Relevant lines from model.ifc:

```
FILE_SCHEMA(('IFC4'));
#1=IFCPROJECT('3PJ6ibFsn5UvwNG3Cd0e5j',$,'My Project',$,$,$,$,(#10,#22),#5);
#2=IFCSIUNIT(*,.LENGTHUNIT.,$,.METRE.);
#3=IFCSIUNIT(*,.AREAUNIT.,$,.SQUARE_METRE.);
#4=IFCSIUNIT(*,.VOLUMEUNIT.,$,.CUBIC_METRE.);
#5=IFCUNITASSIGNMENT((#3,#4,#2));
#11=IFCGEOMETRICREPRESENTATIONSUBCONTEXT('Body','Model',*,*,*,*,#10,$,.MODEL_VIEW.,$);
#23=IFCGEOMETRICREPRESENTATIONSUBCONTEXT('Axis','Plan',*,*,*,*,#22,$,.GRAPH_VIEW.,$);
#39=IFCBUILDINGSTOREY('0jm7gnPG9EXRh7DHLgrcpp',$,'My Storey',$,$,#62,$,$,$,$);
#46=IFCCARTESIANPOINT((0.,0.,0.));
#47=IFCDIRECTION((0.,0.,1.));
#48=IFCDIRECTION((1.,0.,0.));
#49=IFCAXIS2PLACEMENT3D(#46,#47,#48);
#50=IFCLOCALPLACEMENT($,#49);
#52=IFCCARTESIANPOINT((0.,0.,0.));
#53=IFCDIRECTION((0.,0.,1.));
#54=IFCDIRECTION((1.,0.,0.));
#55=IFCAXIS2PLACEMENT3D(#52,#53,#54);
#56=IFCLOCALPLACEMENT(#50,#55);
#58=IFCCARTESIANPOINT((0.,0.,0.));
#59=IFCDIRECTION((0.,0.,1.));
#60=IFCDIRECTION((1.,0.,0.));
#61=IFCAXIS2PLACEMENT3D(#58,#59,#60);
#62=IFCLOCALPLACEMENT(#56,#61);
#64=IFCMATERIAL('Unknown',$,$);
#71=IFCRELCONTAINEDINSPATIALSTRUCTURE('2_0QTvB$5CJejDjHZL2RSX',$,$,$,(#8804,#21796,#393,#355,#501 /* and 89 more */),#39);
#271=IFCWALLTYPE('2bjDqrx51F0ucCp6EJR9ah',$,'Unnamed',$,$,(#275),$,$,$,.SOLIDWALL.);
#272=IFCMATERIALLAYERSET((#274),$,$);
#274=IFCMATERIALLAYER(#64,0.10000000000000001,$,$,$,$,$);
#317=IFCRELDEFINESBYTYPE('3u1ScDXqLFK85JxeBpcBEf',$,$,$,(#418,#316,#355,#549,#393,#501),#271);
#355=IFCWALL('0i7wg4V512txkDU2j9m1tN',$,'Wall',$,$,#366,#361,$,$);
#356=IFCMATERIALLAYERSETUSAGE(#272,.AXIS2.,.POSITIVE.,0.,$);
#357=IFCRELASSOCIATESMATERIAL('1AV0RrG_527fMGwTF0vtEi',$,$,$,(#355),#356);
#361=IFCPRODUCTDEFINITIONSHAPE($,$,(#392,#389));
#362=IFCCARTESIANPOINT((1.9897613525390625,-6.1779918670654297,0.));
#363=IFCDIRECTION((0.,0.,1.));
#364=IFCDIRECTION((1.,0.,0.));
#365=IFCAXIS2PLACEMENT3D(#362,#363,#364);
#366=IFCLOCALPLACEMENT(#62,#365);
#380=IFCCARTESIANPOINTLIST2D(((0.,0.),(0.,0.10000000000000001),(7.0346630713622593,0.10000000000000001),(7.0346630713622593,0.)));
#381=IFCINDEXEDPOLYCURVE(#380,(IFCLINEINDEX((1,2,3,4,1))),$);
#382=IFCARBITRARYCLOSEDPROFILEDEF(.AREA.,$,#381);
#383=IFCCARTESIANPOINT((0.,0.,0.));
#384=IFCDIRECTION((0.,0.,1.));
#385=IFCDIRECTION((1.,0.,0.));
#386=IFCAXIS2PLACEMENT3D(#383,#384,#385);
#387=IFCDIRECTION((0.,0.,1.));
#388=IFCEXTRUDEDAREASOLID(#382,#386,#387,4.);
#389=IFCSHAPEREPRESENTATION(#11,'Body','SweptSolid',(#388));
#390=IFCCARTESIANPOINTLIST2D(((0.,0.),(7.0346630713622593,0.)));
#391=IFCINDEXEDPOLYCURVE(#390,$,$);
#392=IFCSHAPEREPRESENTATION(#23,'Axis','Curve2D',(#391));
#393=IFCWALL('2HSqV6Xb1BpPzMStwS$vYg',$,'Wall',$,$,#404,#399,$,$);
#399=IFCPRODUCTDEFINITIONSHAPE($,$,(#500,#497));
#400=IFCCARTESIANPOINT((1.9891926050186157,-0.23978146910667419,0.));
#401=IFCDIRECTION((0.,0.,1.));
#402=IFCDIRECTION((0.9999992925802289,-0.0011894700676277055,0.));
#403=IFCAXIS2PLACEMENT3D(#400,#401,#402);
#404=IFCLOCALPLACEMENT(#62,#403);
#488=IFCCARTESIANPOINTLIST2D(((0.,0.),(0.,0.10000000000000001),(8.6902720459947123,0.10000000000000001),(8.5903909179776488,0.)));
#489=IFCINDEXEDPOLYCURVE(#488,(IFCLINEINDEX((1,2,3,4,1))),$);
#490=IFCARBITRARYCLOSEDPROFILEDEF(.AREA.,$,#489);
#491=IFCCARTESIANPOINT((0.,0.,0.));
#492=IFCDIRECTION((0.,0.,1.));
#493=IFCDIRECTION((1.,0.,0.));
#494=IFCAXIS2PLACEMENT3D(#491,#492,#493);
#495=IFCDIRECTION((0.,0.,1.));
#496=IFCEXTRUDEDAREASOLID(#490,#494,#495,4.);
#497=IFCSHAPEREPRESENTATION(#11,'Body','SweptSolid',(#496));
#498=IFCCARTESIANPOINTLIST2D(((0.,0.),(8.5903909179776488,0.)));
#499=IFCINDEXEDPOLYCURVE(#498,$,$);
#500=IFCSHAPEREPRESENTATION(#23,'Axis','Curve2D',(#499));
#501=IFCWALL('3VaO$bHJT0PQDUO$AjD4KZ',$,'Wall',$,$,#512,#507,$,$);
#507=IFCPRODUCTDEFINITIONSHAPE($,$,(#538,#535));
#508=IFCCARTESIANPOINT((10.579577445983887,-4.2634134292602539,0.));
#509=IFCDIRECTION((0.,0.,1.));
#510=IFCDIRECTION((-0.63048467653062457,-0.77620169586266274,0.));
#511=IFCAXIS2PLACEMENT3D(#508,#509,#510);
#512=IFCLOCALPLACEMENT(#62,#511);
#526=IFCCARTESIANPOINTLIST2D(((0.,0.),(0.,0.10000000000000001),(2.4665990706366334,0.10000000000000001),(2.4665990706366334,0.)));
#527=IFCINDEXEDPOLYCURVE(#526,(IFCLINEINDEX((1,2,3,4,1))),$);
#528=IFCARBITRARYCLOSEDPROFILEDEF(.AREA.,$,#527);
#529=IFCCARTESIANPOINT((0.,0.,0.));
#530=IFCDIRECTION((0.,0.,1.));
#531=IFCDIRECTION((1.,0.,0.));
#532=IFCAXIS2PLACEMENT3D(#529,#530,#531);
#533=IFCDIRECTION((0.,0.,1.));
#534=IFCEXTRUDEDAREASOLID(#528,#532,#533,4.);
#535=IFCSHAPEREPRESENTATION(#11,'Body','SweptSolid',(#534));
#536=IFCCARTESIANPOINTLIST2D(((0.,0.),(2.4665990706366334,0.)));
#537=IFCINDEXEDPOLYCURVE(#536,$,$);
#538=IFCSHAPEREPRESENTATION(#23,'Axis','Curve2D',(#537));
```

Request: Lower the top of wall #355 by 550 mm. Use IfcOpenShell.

```python
import ifcopenshell
import ifcopenshell.geom
import ifcopenshell.util.representation
import ifcopenshell.util.shape
import ifcopenshell.util.unit

model = ifcopenshell.open("model.ifc")
unit_scale = ifcopenshell.util.unit.calculate_unit_scale(model)
settings = ifcopenshell.geom.settings()


def volume(element):
    """Net volume in cubic metres, openings subtracted."""
    shape = ifcopenshell.geom.create_shape(settings, element)
    return ifcopenshell.util.shape.get_volume(shape.geometry)


wall = model.by_id(355)
before = volume(wall)

body = ifcopenshell.util.representation.get_representation(wall, "Model", "Body")
solid = body.Items[0]
old_height = solid.Depth
solid.Depth -= 0.55 / unit_scale
after = volume(wall)

print(f"height {old_height:g} -> {solid.Depth:g}, volume {before:.3f} -> {after:.3f} m3")

model.write("model-out.ifc")
```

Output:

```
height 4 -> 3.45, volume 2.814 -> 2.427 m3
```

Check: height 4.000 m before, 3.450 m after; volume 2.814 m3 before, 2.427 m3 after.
